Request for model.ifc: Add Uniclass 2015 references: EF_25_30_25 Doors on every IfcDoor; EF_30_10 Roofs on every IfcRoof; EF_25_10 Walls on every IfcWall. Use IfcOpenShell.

First a look at what the model holds.

```python
import ifcopenshell

model = ifcopenshell.open("model.ifc")
print(model.schema)
print("classifications:", [c.Name for c in model.by_type("IfcClassification")])
for ifc_class in ("IfcDoor", "IfcRoof", "IfcStair", "IfcWall", "IfcWindow"):
    print(ifc_class, len(model.by_type(ifc_class)))
```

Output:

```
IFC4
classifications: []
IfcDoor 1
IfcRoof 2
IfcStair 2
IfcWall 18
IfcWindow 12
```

```python
import ifcopenshell
import ifcopenshell.api.classification

model = ifcopenshell.open("model.ifc")

system = ifcopenshell.api.classification.add_classification(model, classification="Uniclass 2015")

codes = {
    "IfcDoor": ("EF_25_30_25", "Doors"),
    "IfcRoof": ("EF_30_10", "Roofs"),
    "IfcWall": ("EF_25_10", "Walls"),
}
for ifc_class, (code, name) in codes.items():
    products = model.by_type(ifc_class)
    ifcopenshell.api.classification.add_reference(
        model, products=products, classification=system, identification=code, name=name
    )
    print(code, len(products))

model.write("model_rev.ifc")
```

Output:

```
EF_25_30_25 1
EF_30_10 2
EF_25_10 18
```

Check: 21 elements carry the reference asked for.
